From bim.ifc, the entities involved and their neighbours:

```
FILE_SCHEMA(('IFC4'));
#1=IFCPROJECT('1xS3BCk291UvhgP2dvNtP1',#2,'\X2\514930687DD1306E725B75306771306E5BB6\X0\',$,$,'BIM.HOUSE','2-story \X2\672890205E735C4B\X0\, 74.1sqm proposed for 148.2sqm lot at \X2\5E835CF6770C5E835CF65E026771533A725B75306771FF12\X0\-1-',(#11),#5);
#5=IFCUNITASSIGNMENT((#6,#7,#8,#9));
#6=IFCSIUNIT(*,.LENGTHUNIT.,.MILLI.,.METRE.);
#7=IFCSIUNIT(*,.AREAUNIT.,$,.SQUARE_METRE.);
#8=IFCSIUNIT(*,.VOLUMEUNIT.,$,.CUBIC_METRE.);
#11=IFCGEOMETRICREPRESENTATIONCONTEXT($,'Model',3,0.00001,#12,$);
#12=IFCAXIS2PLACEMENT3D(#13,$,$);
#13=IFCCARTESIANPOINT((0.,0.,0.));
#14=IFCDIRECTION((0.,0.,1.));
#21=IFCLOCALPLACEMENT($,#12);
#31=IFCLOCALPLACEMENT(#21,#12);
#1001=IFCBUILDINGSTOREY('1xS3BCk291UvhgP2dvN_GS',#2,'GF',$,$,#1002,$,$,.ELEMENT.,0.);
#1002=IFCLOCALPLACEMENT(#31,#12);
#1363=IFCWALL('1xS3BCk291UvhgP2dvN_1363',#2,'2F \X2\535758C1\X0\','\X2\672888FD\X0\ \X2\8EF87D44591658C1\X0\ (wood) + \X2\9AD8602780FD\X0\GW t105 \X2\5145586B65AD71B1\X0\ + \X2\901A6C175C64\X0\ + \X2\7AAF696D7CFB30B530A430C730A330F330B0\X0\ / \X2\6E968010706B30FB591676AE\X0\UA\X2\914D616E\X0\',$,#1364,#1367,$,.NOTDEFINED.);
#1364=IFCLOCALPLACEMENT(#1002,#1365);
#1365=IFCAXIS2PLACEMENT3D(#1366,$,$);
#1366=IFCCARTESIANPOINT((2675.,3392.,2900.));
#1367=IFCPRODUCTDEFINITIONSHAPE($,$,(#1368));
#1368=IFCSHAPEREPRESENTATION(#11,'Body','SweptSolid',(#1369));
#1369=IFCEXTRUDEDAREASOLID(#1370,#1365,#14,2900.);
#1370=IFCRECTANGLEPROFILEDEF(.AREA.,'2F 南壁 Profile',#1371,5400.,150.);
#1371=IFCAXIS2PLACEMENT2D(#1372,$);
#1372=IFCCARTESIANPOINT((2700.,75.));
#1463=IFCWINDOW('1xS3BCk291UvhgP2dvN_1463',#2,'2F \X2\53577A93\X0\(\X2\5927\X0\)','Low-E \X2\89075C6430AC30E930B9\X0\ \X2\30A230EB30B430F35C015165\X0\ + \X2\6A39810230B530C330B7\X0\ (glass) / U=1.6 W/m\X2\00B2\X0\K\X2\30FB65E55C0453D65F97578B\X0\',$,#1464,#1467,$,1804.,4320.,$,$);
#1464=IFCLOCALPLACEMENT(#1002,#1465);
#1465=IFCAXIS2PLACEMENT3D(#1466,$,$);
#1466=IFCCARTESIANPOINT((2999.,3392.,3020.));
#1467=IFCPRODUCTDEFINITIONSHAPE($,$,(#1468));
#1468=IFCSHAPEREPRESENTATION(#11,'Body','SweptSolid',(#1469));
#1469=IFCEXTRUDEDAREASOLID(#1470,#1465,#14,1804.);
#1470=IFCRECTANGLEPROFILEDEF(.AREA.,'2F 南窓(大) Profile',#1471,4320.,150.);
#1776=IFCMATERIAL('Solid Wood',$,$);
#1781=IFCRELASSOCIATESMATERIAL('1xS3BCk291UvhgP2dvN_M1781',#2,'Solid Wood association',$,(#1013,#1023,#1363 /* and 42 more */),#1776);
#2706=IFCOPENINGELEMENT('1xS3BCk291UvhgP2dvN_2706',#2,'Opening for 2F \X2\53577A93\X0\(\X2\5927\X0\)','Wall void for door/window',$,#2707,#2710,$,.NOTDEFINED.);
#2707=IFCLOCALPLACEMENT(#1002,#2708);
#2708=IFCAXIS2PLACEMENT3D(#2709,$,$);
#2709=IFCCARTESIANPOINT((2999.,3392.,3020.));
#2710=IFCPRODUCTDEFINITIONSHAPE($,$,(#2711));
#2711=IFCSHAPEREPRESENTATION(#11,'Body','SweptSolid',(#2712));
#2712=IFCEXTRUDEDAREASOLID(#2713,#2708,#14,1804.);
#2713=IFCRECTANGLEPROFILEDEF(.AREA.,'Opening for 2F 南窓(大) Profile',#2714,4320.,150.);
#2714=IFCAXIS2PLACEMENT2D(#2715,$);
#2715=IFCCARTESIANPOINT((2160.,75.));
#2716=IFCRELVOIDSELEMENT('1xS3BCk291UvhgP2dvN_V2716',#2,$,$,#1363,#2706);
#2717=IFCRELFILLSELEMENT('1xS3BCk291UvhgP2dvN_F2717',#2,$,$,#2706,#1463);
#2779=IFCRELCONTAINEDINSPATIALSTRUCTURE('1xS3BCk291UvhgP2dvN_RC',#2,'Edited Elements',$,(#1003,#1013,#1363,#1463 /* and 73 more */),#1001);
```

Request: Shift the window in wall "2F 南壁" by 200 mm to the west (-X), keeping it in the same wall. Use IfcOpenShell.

```python
import ifcopenshell
import ifcopenshell.api.geometry
import ifcopenshell.util.placement

model = ifcopenshell.open("bim.ifc")

window = model.by_guid("1xS3BCk291UvhgP2dvN_1463")
opening = window.FillsVoids[0].RelatingOpeningElement
wall = opening.VoidsElements[0].RelatingBuildingElement

wall_matrix = ifcopenshell.util.placement.get_local_placement(wall.ObjectPlacement)
shift = wall_matrix[:3, 0] * -200.0
before = ifcopenshell.util.placement.get_local_placement(window.ObjectPlacement)[:3, 3].copy()

# The window is not placed relative to its opening, so move both.
for product in (opening, window):
    matrix = ifcopenshell.util.placement.get_local_placement(product.ObjectPlacement)
    matrix[:3, 3] += shift
    ifcopenshell.api.geometry.edit_object_placement(model, product=product, matrix=matrix, is_si=False)

after = ifcopenshell.util.placement.get_local_placement(window.ObjectPlacement)[:3, 3]
print("window moved by", (after - before).round(3) + 0.0)

model.write("bim_updated.ifc")
```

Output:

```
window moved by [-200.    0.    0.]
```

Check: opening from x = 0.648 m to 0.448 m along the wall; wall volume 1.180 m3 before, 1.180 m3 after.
